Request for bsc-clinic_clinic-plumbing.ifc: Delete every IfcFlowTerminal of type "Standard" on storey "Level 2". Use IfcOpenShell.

First a look at what the model holds.

```python
import ifcopenshell
import ifcopenshell.util.element

model = ifcopenshell.open("bsc-clinic_clinic-plumbing.ifc")
print(model.schema)
storey = next(s for s in model.by_type("IfcBuildingStorey") if s.Name == "Level 2")
terminals = [e for e in ifcopenshell.util.element.get_decomposition(storey) if e.is_a("IfcFlowTerminal")]
seen = {}
for e in terminals:
    element_type = ifcopenshell.util.element.get_type(e)
    name = element_type.Name if element_type not in (None, e) else None
    seen[name] = seen.get(name, 0) + 1
for name, count in sorted(seen.items(), key=str):
    print(count, "x", name)
```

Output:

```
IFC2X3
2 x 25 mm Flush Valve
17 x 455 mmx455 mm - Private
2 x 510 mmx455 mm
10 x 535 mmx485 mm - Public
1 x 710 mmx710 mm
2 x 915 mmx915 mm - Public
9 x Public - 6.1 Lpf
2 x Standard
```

```python
import ifcopenshell
import ifcopenshell.api.root
import ifcopenshell.util.element

model = ifcopenshell.open("bsc-clinic_clinic-plumbing.ifc")

storey = next(s for s in model.by_type("IfcBuildingStorey") if s.Name == "Level 2")
terminals = [e for e in ifcopenshell.util.element.get_decomposition(storey) if e.is_a("IfcFlowTerminal")]
targets = [e for e in terminals if (t := ifcopenshell.util.element.get_type(e)) not in (None, e) and t.Name == "Standard"]

for e in targets:
    ifcopenshell.api.root.remove_product(model, product=e)
print(len(targets), "removed")

model.write("bsc-clinic_clinic-plumbing_v2.ifc")
```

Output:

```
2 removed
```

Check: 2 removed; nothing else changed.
